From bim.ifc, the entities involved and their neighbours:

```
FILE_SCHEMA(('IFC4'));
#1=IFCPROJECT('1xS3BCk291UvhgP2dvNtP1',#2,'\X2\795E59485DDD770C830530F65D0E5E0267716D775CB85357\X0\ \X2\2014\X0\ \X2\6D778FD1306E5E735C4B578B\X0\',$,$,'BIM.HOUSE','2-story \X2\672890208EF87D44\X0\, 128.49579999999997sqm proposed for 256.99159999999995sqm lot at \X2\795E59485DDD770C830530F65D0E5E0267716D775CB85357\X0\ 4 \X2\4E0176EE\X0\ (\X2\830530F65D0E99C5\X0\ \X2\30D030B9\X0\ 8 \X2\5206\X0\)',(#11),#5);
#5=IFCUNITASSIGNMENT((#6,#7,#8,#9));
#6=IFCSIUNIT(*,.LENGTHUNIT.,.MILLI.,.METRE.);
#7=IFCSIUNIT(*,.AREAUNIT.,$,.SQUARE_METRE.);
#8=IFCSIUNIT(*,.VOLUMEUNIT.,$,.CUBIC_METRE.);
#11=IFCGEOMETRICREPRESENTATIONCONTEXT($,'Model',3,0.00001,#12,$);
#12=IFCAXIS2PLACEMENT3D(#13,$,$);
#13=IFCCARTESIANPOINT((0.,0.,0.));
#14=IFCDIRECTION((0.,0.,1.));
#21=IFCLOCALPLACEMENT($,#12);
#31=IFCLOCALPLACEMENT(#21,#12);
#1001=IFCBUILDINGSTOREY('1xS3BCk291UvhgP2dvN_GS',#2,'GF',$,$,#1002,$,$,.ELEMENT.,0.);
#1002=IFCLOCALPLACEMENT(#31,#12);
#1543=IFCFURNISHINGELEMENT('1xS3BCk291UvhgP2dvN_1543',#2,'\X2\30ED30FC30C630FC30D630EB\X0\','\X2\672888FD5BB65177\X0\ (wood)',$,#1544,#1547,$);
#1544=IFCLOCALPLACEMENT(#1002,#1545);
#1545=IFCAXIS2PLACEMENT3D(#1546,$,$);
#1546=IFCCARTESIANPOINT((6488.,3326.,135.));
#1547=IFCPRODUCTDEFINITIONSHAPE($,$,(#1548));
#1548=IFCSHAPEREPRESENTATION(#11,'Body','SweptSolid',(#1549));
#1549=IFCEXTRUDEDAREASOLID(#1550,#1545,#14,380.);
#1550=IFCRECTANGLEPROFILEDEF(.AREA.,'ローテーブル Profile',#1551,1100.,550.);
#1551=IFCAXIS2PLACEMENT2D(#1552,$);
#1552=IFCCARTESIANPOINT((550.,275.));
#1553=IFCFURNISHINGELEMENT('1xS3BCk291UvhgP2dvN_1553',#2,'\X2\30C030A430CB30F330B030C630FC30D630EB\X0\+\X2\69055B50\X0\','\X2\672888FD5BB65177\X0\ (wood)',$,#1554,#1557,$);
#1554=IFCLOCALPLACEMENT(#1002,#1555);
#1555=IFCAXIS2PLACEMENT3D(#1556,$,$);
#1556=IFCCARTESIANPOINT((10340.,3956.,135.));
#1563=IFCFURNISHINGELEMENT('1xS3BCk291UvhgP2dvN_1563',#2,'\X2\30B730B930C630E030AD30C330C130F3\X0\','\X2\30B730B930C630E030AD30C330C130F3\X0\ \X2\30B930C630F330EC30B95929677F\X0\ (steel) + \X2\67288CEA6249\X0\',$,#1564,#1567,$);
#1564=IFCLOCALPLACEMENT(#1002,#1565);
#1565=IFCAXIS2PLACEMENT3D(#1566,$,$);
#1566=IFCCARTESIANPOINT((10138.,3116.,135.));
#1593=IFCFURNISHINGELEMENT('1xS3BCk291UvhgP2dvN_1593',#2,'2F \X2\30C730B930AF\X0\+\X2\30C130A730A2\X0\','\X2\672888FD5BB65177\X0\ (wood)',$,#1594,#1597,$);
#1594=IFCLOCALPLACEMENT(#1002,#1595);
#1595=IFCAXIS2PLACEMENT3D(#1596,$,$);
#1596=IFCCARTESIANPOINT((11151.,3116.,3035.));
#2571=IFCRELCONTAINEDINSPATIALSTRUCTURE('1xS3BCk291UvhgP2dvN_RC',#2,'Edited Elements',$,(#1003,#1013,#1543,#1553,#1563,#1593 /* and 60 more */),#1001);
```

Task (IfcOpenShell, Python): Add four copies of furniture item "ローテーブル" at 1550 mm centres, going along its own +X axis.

```python
import ifcopenshell
import ifcopenshell.api.geometry
import ifcopenshell.api.root
import ifcopenshell.util.element
import ifcopenshell.util.placement
import ifcopenshell.util.unit

model = ifcopenshell.open("bim.ifc")
unit_scale = ifcopenshell.util.unit.calculate_unit_scale(model)


def reuse_history(source, copy):
    """copy_class also copies each property set's owner history, people and application; keep the originals."""
    for rel in copy.IsDefinedBy:
        if rel.is_a("IfcRelDefinesByProperties") and (history := rel.RelatingPropertyDefinition.OwnerHistory):
            rel.RelatingPropertyDefinition.OwnerHistory = source.OwnerHistory
            ifcopenshell.util.element.remove_deep2(model, history)


source = model.by_guid("1xS3BCk291UvhgP2dvN_1543")
base = ifcopenshell.util.placement.get_local_placement(source.ObjectPlacement)
step = base[:3, 0] * 1.55 / unit_scale

for i in range(1, 5):
    copy = ifcopenshell.api.root.copy_class(model, product=source)
    copy.Representation = ifcopenshell.util.element.copy_deep(
        model, source.Representation, exclude=["IfcGeometricRepresentationContext", "IfcRepresentationMap"]
    )
    reuse_history(source, copy)
    matrix = base.copy()
    matrix[:3, 3] += i * step
    print("added at", matrix[:3, 3].round(3) + 0.0)
    ifcopenshell.api.geometry.edit_object_placement(model, product=copy, matrix=matrix, is_si=False)

model.write("bim_v2.ifc")
```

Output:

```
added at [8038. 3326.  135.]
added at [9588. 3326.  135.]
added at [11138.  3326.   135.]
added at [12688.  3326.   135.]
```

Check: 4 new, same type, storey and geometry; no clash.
